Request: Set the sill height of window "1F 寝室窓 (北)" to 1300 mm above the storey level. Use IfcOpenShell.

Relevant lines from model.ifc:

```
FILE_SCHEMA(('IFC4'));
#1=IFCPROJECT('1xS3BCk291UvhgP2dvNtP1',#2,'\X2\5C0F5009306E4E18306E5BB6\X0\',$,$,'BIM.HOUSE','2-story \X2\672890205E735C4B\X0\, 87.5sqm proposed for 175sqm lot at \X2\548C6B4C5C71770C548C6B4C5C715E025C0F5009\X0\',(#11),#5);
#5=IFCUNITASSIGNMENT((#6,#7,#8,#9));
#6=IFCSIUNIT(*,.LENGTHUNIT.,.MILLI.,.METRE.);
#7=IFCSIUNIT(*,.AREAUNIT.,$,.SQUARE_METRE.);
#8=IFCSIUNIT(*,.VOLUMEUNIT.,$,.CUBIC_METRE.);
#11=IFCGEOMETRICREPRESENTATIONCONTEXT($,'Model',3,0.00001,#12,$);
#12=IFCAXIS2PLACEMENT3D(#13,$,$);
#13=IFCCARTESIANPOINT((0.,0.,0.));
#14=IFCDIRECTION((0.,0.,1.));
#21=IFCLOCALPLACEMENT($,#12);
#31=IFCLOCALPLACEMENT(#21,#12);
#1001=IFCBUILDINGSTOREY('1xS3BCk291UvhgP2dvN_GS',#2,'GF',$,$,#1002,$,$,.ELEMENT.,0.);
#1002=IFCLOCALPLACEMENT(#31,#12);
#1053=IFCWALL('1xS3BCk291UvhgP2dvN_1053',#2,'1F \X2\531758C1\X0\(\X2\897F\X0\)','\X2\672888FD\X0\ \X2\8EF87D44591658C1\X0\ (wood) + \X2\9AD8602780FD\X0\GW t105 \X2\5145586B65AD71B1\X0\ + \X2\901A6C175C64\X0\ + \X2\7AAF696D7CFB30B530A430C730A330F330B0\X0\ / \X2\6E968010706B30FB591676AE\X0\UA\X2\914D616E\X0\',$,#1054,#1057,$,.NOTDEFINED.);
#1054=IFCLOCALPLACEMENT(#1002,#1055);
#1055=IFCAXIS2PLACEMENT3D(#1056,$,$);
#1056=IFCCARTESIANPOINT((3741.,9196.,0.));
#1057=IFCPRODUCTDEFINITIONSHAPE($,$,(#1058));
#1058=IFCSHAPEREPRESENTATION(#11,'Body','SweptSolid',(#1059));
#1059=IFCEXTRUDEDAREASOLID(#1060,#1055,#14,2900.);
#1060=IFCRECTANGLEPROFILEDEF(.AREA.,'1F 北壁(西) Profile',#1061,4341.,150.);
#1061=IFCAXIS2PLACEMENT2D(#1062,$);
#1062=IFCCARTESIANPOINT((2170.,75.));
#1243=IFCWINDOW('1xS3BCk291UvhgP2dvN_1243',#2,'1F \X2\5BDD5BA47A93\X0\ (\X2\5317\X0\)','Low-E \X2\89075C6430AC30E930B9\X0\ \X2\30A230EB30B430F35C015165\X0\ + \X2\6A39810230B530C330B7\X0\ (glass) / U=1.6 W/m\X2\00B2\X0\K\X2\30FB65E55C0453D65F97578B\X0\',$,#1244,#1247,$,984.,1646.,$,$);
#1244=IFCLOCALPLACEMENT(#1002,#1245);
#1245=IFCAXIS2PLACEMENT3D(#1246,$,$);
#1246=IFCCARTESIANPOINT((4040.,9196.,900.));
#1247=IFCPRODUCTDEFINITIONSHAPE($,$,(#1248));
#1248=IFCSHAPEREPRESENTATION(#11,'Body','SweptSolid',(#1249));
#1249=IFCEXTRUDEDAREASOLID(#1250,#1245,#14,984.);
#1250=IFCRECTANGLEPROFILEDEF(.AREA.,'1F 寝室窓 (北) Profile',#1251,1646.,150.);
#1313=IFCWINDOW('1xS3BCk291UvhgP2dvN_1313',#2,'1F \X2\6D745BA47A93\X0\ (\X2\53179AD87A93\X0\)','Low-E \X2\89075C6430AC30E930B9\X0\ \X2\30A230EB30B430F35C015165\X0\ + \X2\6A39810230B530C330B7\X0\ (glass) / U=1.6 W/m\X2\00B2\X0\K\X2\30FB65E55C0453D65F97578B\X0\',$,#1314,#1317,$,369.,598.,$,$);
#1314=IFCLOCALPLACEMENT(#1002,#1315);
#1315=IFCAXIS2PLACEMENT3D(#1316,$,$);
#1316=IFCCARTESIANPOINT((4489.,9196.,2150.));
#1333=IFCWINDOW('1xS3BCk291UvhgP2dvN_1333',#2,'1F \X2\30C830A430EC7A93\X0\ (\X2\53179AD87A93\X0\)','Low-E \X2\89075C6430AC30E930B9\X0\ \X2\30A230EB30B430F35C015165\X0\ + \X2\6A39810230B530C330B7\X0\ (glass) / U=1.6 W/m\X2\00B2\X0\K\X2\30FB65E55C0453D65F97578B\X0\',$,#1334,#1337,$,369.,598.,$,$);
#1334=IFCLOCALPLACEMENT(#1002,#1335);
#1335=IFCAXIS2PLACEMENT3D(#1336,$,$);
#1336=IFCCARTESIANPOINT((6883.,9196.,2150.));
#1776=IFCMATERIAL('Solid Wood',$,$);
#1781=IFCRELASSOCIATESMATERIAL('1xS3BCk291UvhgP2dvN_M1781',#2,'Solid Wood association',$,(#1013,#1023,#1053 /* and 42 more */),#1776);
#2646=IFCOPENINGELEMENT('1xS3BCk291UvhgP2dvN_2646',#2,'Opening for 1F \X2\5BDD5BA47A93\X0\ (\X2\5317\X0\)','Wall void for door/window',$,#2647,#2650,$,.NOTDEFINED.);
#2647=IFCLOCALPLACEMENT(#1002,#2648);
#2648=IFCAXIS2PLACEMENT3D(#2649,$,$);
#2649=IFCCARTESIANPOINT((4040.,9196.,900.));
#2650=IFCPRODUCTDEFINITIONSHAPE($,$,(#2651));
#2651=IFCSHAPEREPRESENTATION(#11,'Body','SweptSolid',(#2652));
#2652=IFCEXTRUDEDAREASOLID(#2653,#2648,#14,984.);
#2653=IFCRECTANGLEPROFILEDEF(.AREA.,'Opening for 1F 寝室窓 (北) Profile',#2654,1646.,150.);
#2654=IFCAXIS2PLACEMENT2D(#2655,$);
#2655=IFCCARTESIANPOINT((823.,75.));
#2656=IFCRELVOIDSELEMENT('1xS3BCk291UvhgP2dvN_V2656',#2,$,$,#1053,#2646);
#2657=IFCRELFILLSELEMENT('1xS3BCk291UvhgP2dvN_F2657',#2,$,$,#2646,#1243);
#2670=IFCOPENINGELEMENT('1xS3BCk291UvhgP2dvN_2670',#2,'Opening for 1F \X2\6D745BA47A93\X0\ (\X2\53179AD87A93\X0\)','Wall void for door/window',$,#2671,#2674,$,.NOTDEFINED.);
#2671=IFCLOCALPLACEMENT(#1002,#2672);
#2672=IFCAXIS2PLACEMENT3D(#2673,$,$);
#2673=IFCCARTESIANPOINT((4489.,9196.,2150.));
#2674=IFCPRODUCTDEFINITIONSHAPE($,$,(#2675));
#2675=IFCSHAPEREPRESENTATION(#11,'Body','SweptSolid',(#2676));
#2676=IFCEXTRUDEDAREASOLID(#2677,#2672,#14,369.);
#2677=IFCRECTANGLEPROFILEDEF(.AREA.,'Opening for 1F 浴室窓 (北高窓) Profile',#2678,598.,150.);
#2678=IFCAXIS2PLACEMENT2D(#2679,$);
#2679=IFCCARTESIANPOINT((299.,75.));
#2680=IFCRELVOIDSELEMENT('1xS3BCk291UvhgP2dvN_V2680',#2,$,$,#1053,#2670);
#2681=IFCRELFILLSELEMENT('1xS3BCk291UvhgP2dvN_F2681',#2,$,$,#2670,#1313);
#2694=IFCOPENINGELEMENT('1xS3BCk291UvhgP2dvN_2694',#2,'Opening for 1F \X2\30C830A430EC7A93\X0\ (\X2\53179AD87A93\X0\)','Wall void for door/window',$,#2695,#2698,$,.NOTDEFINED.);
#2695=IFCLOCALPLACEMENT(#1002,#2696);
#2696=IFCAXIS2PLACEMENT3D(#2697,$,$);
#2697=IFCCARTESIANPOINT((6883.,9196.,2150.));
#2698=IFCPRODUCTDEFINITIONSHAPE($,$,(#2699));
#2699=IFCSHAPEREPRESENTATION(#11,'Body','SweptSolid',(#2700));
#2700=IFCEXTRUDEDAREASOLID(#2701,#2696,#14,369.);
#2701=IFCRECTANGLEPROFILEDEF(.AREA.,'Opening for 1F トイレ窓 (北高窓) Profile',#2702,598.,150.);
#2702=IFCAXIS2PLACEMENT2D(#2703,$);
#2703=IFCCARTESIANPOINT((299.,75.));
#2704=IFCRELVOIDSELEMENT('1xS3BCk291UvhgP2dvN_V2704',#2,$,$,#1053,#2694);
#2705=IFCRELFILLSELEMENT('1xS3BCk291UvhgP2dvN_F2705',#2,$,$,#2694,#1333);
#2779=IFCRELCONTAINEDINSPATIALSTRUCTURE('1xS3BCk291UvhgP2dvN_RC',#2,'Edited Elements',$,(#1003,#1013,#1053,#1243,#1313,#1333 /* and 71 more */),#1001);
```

```python
import numpy as np
import ifcopenshell
import ifcopenshell.api.geometry
import ifcopenshell.geom
import ifcopenshell.util.element
import ifcopenshell.util.placement
import ifcopenshell.util.shape
import ifcopenshell.util.unit

model = ifcopenshell.open("model.ifc")
unit_scale = ifcopenshell.util.unit.calculate_unit_scale(model)

window = model.by_guid("1xS3BCk291UvhgP2dvN_1243")
opening = window.FillsVoids[0].RelatingOpeningElement
storey = ifcopenshell.util.element.get_container(window, ifc_class="IfcBuildingStorey")
level = ifcopenshell.util.placement.get_local_placement(storey.ObjectPlacement)[2, 3]

# The opening's origin need not be at the sill, so measure its lowest point.
shape = ifcopenshell.geom.create_shape(ifcopenshell.geom.settings(), opening)
bottom = ifcopenshell.util.shape.get_shape_bottom_elevation(shape, shape.geometry) / unit_scale
dz = level + 1300.0 - bottom

shift = np.array([0.0, 0.0, dz])
# The window is not placed relative to its opening, so move both.
for product in (opening, window):
    matrix = ifcopenshell.util.placement.get_local_placement(product.ObjectPlacement)
    matrix[:3, 3] += shift
    ifcopenshell.api.geometry.edit_object_placement(model, product=product, matrix=matrix, is_si=False)

print(f"moved by {dz * unit_scale:+.3f} m")

model.write("model_updated.ifc")
```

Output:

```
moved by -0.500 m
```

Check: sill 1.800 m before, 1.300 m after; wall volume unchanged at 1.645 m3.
